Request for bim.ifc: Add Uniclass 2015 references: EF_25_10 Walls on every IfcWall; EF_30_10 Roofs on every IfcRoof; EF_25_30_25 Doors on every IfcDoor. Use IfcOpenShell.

First a look at what the model holds.

```python
import ifcopenshell

model = ifcopenshell.open("bim.ifc")
print(model.schema)
print("classifications:", [c.Name for c in model.by_type("IfcClassification")])
for ifc_class in ("IfcDoor", "IfcRoof", "IfcStair", "IfcWall", "IfcWindow"):
    print(ifc_class, len(model.by_type(ifc_class)))
```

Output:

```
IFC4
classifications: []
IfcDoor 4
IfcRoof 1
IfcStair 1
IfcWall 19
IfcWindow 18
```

```python
import ifcopenshell
import ifcopenshell.api.classification

model = ifcopenshell.open("bim.ifc")

system = ifcopenshell.api.classification.add_classification(model, classification="Uniclass 2015")

codes = {
    "IfcWall": ("EF_25_10", "Walls"),
    "IfcRoof": ("EF_30_10", "Roofs"),
    "IfcDoor": ("EF_25_30_25", "Doors"),
}
for ifc_class, (code, name) in codes.items():
    products = model.by_type(ifc_class)
    ifcopenshell.api.classification.add_reference(
        model, products=products, classification=system, identification=code, name=name
    )
    print(code, len(products))

model.write("bim_updated.ifc")
```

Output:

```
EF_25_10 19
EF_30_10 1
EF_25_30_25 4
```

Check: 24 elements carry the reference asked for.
